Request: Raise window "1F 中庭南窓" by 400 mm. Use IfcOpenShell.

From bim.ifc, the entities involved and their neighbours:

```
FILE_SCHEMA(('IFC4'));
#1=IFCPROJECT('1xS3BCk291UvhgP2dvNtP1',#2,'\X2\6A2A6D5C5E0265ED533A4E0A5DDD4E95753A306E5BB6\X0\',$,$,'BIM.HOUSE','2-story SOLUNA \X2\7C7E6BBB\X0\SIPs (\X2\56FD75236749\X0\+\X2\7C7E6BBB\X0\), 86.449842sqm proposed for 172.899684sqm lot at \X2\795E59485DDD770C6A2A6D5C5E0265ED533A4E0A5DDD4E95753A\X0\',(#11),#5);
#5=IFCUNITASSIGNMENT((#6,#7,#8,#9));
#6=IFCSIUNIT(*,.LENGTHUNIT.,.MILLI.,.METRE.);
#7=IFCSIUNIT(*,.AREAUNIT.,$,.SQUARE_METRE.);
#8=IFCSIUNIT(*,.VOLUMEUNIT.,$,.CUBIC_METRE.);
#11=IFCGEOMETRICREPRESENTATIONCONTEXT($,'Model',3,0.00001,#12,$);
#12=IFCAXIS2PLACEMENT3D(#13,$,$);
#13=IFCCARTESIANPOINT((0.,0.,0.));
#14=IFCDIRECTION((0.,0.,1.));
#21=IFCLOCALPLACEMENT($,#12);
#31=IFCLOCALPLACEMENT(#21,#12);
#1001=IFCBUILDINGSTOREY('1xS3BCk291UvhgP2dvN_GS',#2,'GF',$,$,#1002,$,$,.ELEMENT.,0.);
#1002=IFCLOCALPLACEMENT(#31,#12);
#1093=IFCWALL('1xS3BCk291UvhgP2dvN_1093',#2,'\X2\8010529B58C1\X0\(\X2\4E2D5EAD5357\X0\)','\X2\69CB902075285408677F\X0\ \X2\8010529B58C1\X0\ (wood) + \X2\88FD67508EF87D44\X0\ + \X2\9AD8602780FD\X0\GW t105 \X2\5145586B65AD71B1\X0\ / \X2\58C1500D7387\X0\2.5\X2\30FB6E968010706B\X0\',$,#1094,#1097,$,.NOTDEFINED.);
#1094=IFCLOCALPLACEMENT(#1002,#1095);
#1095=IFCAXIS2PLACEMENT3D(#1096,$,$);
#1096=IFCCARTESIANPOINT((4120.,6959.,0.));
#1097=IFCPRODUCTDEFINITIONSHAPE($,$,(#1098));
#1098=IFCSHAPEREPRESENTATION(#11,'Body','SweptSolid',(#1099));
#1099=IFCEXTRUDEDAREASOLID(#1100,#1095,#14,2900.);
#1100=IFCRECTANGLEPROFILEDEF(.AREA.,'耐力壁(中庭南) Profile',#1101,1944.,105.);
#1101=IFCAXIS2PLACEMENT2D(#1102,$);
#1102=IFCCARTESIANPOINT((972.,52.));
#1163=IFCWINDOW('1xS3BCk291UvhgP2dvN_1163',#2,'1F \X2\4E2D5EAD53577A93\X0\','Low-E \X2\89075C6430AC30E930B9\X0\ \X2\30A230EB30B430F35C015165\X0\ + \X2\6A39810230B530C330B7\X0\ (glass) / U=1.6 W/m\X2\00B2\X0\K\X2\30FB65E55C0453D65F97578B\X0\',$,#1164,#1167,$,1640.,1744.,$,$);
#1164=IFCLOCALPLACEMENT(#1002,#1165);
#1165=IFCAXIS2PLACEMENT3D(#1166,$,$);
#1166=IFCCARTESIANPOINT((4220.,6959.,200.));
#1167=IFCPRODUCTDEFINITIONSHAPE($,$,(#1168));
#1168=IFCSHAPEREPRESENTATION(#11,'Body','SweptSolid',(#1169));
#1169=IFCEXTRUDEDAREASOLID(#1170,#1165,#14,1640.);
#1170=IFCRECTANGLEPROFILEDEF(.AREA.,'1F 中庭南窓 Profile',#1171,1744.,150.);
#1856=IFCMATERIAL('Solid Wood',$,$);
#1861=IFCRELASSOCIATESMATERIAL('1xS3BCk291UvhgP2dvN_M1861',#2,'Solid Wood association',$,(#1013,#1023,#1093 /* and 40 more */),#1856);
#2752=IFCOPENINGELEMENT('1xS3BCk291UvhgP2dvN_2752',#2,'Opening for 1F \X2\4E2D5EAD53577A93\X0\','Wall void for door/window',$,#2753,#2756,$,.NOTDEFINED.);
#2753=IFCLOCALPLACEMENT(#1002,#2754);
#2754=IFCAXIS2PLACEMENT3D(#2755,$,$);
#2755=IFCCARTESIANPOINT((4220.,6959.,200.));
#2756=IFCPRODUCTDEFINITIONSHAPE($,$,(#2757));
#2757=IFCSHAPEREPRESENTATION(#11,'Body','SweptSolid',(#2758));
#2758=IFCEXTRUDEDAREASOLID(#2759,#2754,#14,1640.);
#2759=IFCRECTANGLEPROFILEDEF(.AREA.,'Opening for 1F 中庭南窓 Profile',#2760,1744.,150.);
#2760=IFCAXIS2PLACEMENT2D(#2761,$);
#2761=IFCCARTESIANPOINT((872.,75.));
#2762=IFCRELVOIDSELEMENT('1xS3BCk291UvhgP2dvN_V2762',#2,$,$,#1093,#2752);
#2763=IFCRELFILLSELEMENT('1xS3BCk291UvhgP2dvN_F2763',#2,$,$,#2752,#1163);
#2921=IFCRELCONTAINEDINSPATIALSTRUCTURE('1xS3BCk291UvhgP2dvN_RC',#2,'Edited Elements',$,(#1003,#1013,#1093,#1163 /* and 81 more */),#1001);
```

```python
import numpy as np
import ifcopenshell
import ifcopenshell.api.geometry
import ifcopenshell.util.placement
import ifcopenshell.util.unit

model = ifcopenshell.open("bim.ifc")
unit_scale = ifcopenshell.util.unit.calculate_unit_scale(model)

window = model.by_id(1163)
opening = window.FillsVoids[0].RelatingOpeningElement
dz = 400.0

shift = np.array([0.0, 0.0, dz])
# The window is not placed relative to its opening, so move both.
for product in (opening, window):
    matrix = ifcopenshell.util.placement.get_local_placement(product.ObjectPlacement)
    matrix[:3, 3] += shift
    ifcopenshell.api.geometry.edit_object_placement(model, product=product, matrix=matrix, is_si=False)

print(f"moved by {dz * unit_scale:+.3f} m")

model.write("bim_edited.ifc")
```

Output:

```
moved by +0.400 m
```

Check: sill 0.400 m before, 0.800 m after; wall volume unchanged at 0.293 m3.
